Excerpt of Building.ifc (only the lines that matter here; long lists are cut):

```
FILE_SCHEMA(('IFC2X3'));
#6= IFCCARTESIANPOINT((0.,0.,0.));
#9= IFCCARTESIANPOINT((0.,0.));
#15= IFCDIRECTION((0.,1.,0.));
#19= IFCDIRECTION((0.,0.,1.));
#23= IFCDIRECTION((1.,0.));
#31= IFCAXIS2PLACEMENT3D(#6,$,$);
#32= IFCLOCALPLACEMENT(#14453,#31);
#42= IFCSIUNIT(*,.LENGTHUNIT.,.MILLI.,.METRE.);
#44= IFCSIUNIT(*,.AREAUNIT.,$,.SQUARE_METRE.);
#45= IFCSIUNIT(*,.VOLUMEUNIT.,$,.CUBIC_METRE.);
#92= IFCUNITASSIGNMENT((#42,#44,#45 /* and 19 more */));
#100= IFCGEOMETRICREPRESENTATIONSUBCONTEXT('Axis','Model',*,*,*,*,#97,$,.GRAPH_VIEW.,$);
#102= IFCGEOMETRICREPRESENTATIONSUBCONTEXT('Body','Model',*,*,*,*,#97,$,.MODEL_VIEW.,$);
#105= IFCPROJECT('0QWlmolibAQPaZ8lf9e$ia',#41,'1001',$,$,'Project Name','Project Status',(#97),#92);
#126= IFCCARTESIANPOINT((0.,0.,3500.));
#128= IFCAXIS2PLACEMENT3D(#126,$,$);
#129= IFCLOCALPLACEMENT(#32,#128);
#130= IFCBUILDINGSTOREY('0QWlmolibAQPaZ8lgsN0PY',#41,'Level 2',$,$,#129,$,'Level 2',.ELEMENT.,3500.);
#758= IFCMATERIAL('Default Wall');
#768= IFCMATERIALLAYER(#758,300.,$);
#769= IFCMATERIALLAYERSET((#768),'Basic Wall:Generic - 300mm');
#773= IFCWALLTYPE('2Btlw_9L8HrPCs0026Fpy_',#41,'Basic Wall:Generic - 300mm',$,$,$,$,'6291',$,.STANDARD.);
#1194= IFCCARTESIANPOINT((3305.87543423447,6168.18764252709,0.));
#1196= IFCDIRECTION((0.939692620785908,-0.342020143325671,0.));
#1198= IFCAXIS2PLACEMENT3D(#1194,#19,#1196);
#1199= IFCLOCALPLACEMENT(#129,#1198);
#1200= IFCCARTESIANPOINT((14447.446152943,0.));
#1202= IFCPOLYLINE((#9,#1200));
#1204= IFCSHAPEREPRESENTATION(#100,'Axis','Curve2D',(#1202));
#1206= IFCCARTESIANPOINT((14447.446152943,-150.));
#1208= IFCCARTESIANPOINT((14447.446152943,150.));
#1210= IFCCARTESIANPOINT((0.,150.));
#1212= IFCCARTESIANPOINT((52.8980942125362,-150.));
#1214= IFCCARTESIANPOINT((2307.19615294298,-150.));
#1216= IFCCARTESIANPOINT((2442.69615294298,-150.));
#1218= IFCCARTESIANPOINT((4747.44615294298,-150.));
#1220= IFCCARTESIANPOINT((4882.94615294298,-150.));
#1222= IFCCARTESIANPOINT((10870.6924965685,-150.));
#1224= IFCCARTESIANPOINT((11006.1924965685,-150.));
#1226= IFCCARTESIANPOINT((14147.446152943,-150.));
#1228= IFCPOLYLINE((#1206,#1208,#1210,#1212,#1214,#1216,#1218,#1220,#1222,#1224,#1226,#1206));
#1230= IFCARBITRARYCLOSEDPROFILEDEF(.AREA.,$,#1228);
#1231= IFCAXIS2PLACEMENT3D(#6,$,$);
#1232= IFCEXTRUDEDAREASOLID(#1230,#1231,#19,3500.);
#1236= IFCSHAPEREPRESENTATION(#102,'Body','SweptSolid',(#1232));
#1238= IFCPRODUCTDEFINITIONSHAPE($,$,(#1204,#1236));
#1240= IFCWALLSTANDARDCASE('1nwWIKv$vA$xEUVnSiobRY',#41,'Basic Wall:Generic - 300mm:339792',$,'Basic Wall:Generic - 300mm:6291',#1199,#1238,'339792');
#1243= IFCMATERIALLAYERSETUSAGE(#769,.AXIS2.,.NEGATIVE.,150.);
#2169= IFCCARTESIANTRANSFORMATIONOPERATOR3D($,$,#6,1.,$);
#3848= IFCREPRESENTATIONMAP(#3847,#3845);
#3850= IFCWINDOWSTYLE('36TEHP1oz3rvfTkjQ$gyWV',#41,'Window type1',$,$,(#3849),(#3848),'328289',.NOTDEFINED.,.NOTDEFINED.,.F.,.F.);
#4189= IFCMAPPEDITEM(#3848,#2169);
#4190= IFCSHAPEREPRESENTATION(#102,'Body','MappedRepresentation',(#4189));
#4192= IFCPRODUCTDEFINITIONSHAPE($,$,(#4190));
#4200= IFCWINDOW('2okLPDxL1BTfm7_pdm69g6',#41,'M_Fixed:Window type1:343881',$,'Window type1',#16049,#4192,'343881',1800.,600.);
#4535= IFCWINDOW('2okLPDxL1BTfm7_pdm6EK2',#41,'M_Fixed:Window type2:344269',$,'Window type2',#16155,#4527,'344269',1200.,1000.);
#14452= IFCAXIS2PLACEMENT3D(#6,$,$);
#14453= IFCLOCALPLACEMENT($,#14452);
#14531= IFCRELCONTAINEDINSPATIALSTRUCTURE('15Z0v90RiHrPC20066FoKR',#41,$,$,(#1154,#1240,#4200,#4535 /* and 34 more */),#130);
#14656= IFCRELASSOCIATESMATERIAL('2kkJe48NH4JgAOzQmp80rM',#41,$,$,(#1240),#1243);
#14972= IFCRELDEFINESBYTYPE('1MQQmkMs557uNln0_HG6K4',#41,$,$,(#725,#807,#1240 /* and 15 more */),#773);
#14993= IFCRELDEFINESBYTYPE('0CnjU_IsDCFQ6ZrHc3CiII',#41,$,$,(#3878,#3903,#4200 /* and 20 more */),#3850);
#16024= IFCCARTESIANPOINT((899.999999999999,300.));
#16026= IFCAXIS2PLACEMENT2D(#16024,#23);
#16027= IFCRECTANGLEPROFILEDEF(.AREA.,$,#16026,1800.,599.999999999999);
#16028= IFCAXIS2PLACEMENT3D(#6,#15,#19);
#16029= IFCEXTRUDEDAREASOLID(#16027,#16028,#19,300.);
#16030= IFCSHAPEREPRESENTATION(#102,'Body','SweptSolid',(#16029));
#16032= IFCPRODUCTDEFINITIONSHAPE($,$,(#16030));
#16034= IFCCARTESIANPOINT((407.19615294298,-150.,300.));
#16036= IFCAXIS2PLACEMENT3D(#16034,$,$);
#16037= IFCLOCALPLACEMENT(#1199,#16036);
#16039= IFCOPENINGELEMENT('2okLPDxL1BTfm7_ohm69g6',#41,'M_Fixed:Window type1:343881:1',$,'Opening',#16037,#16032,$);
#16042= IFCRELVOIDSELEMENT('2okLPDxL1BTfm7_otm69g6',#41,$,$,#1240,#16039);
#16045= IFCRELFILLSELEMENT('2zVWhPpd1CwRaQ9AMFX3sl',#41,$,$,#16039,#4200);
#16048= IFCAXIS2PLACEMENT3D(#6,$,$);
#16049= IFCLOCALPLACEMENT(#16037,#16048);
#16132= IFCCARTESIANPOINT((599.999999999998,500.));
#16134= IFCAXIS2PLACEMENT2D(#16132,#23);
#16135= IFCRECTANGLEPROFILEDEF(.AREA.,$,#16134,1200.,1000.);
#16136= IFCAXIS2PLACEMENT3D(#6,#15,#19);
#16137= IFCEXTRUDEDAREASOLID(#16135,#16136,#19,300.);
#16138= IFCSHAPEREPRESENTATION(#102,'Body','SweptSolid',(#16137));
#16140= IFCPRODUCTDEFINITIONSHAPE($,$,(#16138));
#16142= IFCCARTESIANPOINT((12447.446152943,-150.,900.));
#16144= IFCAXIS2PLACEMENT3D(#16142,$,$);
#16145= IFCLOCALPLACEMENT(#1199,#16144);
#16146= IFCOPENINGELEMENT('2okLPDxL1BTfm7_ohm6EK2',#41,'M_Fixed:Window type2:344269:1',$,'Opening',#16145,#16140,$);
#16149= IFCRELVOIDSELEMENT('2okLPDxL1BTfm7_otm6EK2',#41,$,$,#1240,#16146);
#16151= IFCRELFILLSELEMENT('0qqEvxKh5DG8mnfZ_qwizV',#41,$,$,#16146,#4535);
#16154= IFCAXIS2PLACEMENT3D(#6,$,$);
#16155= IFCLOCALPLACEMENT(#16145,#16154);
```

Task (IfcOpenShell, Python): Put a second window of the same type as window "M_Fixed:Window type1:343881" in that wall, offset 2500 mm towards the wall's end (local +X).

```python
import ifcopenshell
import ifcopenshell.api.feature
import ifcopenshell.api.geometry
import ifcopenshell.api.root
import ifcopenshell.geom
import ifcopenshell.util.element
import ifcopenshell.util.placement
import ifcopenshell.util.shape
import ifcopenshell.util.unit

model = ifcopenshell.open("Building.ifc")
unit_scale = ifcopenshell.util.unit.calculate_unit_scale(model)
settings = ifcopenshell.geom.settings()


def volume(element):
    """Net volume in cubic metres, openings subtracted."""
    shape = ifcopenshell.geom.create_shape(settings, element)
    return ifcopenshell.util.shape.get_volume(shape.geometry)


def reuse_history(source, copy):
    """copy_class also copies each property set's owner history, people and application; keep the originals."""
    for rel in copy.IsDefinedBy:
        if rel.is_a("IfcRelDefinesByProperties") and (history := rel.RelatingPropertyDefinition.OwnerHistory):
            rel.RelatingPropertyDefinition.OwnerHistory = source.OwnerHistory
            ifcopenshell.util.element.remove_deep2(model, history)


window = model.by_guid("2okLPDxL1BTfm7_pdm69g6")
opening = window.FillsVoids[0].RelatingOpeningElement
wall = opening.VoidsElements[0].RelatingBuildingElement
before = volume(wall)
shift = ifcopenshell.util.placement.get_local_placement(wall.ObjectPlacement)[:3, 0] * 2.5 / unit_scale

# copy_class copies the void relationship, type, container and properties, but no geometry.
new_opening = ifcopenshell.api.root.copy_class(model, product=opening)
new_opening.Representation = ifcopenshell.util.element.copy_deep(
    model, opening.Representation, exclude=["IfcGeometricRepresentationContext", "IfcRepresentationMap"]
)
new_opening.Name = "M_Fixed:Window type1"
new_window = ifcopenshell.api.root.copy_class(model, product=window)
new_window.Representation = ifcopenshell.util.element.copy_deep(
    model, window.Representation, exclude=["IfcGeometricRepresentationContext", "IfcRepresentationMap"]
)
new_window.Name = "M_Fixed:Window type1"
new_window.Tag = None
reuse_history(window, new_window)
fills = ifcopenshell.api.feature.add_filling(model, opening=new_opening, element=new_window)
fills.OwnerHistory = new_window.OwnerHistory  # required in IFC2X3

for old, new in ((opening, new_opening), (window, new_window)):
    matrix = ifcopenshell.util.placement.get_local_placement(old.ObjectPlacement)
    matrix[:3, 3] += shift
    ifcopenshell.api.geometry.edit_object_placement(model, product=new, matrix=matrix, is_si=False)

after = volume(wall)

print(f"wall volume {before:.3f} -> {after:.3f} m3")

model.write("Building_updated.ifc")
```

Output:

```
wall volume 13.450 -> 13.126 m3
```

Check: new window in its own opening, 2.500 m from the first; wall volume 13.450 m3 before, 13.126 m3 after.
